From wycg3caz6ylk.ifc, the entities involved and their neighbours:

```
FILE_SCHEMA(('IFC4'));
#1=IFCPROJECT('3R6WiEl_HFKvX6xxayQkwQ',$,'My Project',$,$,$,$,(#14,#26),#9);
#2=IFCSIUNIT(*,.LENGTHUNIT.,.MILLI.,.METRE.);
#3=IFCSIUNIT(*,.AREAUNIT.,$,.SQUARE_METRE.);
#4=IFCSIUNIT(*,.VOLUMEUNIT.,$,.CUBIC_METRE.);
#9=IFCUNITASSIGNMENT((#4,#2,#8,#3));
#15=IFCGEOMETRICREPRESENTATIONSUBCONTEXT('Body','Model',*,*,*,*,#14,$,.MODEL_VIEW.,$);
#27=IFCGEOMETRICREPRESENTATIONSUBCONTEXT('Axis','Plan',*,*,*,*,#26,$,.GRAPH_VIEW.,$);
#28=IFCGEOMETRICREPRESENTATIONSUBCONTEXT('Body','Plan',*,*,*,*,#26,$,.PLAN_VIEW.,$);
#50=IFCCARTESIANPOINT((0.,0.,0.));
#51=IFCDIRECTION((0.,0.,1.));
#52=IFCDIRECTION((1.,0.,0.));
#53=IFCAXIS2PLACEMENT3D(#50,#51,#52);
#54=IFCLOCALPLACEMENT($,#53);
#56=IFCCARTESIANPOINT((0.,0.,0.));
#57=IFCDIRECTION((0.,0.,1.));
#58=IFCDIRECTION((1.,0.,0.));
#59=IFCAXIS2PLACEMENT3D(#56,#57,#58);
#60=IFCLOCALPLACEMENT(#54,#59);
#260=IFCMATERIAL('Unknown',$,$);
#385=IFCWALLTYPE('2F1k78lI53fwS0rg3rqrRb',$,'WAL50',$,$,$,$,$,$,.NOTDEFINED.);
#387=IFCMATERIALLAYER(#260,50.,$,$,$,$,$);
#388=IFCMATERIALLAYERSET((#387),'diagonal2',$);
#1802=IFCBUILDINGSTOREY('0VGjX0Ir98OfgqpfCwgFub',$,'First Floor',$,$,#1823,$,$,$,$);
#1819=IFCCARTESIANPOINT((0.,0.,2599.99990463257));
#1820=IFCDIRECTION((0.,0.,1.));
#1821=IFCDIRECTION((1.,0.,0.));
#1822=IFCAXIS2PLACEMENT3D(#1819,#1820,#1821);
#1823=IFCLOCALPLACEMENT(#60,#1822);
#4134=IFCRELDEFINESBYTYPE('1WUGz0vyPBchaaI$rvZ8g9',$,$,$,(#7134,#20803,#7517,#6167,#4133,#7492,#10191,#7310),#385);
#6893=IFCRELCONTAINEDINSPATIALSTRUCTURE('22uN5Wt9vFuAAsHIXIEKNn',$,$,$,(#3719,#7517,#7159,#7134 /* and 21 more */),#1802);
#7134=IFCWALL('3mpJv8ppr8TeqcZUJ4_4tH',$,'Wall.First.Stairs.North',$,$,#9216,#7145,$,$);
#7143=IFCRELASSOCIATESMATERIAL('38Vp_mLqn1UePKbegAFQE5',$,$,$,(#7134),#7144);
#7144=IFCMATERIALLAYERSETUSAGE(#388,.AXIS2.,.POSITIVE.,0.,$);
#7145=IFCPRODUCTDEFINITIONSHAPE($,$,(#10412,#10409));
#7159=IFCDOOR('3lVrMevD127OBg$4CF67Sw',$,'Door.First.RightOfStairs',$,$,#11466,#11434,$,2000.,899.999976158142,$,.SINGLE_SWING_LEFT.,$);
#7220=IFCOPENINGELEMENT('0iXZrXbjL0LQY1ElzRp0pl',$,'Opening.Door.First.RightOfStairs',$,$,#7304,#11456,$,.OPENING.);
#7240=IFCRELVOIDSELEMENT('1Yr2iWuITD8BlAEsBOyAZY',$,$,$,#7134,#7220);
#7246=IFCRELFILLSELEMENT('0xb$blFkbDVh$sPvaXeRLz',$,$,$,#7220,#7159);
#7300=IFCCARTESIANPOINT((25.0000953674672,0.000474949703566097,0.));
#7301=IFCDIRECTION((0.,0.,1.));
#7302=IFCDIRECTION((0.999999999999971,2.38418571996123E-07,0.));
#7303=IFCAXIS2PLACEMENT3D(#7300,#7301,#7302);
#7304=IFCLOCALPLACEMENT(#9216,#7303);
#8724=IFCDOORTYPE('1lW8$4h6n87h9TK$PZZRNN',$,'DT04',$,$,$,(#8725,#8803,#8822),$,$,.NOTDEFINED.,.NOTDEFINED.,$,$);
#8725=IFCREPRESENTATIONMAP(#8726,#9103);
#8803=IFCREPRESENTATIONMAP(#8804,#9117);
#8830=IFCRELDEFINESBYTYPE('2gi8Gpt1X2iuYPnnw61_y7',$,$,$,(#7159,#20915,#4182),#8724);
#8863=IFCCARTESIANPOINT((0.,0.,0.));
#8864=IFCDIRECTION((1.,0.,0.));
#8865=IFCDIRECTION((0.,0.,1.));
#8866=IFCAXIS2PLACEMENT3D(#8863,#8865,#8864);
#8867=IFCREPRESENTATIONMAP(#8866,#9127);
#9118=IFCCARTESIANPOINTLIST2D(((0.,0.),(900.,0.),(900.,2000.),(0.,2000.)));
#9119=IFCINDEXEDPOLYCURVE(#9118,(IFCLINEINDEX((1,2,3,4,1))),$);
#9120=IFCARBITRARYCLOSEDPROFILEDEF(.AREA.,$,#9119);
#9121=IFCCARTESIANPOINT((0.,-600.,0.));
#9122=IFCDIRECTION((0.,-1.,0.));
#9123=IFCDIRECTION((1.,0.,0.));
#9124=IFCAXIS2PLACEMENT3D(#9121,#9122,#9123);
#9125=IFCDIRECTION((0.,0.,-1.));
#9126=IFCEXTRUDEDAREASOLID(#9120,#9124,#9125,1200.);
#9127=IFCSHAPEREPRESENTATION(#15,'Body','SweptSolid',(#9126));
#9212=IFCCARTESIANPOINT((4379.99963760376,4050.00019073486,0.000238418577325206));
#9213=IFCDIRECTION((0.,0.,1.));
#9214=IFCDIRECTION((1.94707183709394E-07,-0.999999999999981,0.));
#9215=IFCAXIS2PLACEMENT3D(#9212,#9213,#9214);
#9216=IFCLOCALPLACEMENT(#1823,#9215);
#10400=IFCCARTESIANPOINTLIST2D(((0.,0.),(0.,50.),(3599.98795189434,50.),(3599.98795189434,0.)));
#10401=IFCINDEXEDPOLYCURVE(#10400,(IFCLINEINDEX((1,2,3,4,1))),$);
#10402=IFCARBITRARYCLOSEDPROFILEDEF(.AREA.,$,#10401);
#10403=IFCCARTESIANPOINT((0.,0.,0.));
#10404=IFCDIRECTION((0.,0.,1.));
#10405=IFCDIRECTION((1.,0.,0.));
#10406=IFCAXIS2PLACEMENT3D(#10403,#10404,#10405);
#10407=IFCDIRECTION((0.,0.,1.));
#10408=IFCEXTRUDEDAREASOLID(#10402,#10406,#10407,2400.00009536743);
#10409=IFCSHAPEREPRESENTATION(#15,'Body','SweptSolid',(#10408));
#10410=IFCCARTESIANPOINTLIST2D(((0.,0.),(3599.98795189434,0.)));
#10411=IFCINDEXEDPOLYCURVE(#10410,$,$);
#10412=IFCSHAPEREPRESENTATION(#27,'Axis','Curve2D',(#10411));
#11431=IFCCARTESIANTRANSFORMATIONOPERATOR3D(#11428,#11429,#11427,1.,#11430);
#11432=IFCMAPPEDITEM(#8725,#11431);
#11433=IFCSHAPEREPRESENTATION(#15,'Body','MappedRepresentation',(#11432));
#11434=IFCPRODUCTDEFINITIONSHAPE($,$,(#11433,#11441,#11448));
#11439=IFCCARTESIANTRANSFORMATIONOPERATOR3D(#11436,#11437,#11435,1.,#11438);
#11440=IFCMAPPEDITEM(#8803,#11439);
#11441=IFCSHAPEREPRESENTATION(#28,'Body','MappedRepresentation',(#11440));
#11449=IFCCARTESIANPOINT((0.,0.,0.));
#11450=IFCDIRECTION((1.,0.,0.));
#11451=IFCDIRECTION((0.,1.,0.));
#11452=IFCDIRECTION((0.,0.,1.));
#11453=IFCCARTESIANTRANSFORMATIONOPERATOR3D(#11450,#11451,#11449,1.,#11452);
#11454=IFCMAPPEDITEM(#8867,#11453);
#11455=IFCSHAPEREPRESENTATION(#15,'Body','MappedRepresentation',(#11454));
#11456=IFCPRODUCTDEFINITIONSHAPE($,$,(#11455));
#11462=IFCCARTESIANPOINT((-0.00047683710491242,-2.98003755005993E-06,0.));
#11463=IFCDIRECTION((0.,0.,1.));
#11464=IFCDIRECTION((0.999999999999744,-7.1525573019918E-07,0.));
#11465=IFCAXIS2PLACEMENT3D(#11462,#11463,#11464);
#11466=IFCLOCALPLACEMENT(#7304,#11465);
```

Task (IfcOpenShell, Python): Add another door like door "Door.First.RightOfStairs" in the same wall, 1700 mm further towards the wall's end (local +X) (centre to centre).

```python
import ifcopenshell
import ifcopenshell.api.feature
import ifcopenshell.api.geometry
import ifcopenshell.api.root
import ifcopenshell.geom
import ifcopenshell.util.element
import ifcopenshell.util.placement
import ifcopenshell.util.shape
import ifcopenshell.util.unit

model = ifcopenshell.open("wycg3caz6ylk.ifc")
unit_scale = ifcopenshell.util.unit.calculate_unit_scale(model)
settings = ifcopenshell.geom.settings()


def volume(element):
    """Net volume in cubic metres, openings subtracted."""
    shape = ifcopenshell.geom.create_shape(settings, element)
    return ifcopenshell.util.shape.get_volume(shape.geometry)


door = model.by_guid("3lVrMevD127OBg$4CF67Sw")
opening = door.FillsVoids[0].RelatingOpeningElement
wall = opening.VoidsElements[0].RelatingBuildingElement
before = volume(wall)
shift = ifcopenshell.util.placement.get_local_placement(wall.ObjectPlacement)[:3, 0] * 1.7 / unit_scale

# copy_class copies the void relationship, type, container and properties, but no geometry.
new_opening = ifcopenshell.api.root.copy_class(model, product=opening)
new_opening.Representation = ifcopenshell.util.element.copy_deep(
    model, opening.Representation, exclude=["IfcGeometricRepresentationContext", "IfcRepresentationMap"]
)
new_door = ifcopenshell.api.root.copy_class(model, product=door)
new_door.Representation = ifcopenshell.util.element.copy_deep(
    model, door.Representation, exclude=["IfcGeometricRepresentationContext", "IfcRepresentationMap"]
)
ifcopenshell.api.feature.add_filling(model, opening=new_opening, element=new_door)

for old, new in ((opening, new_opening), (door, new_door)):
    matrix = ifcopenshell.util.placement.get_local_placement(old.ObjectPlacement)
    matrix[:3, 3] += shift
    ifcopenshell.api.geometry.edit_object_placement(model, product=new, matrix=matrix, is_si=False)

after = volume(wall)

print(f"wall volume {before:.3f} -> {after:.3f} m3")

model.write("wycg3caz6ylk_updated.ifc")
```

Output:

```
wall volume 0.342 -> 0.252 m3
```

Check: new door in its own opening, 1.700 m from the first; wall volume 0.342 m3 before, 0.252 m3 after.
